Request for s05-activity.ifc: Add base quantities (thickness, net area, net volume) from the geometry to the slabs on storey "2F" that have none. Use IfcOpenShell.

First a look at what the model holds.

```python
import ifcopenshell
import ifcopenshell.util.element
import ifcopenshell.util.unit

model = ifcopenshell.open("s05-activity.ifc")
print(model.schema)
for unit_type in ("LENGTHUNIT", "AREAUNIT", "VOLUMEUNIT"):
    print(unit_type, ifcopenshell.util.unit.calculate_unit_scale(model, unit_type))
storey = next(s for s in model.by_type("IfcBuildingStorey") if s.Name == "2F")
slabs = [e for e in ifcopenshell.util.element.get_decomposition(storey) if e.is_a("IfcSlab")]
for e in sorted(slabs, key=lambda e: e.id()):
    print(e.id(), e.is_a(), e.Name, list(ifcopenshell.util.element.get_psets(e, qtos_only=True)), sep=" | ")
```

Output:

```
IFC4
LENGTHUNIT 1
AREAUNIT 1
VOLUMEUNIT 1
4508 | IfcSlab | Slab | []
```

```python
import ifcopenshell
import ifcopenshell.api.pset
import ifcopenshell.geom
import ifcopenshell.util.element
import ifcopenshell.util.shape
import ifcopenshell.util.unit

model = ifcopenshell.open("s05-activity.ifc")
unit_scale = ifcopenshell.util.unit.calculate_unit_scale(model)
area_scale = ifcopenshell.util.unit.calculate_unit_scale(model, "AREAUNIT")
volume_scale = ifcopenshell.util.unit.calculate_unit_scale(model, "VOLUMEUNIT")
settings = ifcopenshell.geom.settings()

storey = next(s for s in model.by_type("IfcBuildingStorey") if s.Name == "2F")
slabs = [e for e in ifcopenshell.util.element.get_decomposition(storey) if e.is_a("IfcSlab")]

for e in sorted(slabs, key=lambda e: e.id()):
    if ifcopenshell.util.element.get_psets(e, qtos_only=True, should_inherit=False):
        continue
    # Geometry comes back in metres, in the element's own axes.
    shape = ifcopenshell.geom.create_shape(settings, e)
    values = {
        "Width": ifcopenshell.util.shape.get_z(shape.geometry) / unit_scale,
        "NetArea": ifcopenshell.util.shape.get_footprint_area(shape.geometry) / area_scale,
        "NetVolume": ifcopenshell.util.shape.get_volume(shape.geometry) / volume_scale,
    }
    qto = ifcopenshell.api.pset.add_qto(model, product=e, name="Qto_SlabBaseQuantities")
    ifcopenshell.api.pset.edit_qto(model, qto=qto, properties=values)
    print(e.id(), {k: round(v, 3) for k, v in values.items()})

model.write("s05-activity-out.ifc")
```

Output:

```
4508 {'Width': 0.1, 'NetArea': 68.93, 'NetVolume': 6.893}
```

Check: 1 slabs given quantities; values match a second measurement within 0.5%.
